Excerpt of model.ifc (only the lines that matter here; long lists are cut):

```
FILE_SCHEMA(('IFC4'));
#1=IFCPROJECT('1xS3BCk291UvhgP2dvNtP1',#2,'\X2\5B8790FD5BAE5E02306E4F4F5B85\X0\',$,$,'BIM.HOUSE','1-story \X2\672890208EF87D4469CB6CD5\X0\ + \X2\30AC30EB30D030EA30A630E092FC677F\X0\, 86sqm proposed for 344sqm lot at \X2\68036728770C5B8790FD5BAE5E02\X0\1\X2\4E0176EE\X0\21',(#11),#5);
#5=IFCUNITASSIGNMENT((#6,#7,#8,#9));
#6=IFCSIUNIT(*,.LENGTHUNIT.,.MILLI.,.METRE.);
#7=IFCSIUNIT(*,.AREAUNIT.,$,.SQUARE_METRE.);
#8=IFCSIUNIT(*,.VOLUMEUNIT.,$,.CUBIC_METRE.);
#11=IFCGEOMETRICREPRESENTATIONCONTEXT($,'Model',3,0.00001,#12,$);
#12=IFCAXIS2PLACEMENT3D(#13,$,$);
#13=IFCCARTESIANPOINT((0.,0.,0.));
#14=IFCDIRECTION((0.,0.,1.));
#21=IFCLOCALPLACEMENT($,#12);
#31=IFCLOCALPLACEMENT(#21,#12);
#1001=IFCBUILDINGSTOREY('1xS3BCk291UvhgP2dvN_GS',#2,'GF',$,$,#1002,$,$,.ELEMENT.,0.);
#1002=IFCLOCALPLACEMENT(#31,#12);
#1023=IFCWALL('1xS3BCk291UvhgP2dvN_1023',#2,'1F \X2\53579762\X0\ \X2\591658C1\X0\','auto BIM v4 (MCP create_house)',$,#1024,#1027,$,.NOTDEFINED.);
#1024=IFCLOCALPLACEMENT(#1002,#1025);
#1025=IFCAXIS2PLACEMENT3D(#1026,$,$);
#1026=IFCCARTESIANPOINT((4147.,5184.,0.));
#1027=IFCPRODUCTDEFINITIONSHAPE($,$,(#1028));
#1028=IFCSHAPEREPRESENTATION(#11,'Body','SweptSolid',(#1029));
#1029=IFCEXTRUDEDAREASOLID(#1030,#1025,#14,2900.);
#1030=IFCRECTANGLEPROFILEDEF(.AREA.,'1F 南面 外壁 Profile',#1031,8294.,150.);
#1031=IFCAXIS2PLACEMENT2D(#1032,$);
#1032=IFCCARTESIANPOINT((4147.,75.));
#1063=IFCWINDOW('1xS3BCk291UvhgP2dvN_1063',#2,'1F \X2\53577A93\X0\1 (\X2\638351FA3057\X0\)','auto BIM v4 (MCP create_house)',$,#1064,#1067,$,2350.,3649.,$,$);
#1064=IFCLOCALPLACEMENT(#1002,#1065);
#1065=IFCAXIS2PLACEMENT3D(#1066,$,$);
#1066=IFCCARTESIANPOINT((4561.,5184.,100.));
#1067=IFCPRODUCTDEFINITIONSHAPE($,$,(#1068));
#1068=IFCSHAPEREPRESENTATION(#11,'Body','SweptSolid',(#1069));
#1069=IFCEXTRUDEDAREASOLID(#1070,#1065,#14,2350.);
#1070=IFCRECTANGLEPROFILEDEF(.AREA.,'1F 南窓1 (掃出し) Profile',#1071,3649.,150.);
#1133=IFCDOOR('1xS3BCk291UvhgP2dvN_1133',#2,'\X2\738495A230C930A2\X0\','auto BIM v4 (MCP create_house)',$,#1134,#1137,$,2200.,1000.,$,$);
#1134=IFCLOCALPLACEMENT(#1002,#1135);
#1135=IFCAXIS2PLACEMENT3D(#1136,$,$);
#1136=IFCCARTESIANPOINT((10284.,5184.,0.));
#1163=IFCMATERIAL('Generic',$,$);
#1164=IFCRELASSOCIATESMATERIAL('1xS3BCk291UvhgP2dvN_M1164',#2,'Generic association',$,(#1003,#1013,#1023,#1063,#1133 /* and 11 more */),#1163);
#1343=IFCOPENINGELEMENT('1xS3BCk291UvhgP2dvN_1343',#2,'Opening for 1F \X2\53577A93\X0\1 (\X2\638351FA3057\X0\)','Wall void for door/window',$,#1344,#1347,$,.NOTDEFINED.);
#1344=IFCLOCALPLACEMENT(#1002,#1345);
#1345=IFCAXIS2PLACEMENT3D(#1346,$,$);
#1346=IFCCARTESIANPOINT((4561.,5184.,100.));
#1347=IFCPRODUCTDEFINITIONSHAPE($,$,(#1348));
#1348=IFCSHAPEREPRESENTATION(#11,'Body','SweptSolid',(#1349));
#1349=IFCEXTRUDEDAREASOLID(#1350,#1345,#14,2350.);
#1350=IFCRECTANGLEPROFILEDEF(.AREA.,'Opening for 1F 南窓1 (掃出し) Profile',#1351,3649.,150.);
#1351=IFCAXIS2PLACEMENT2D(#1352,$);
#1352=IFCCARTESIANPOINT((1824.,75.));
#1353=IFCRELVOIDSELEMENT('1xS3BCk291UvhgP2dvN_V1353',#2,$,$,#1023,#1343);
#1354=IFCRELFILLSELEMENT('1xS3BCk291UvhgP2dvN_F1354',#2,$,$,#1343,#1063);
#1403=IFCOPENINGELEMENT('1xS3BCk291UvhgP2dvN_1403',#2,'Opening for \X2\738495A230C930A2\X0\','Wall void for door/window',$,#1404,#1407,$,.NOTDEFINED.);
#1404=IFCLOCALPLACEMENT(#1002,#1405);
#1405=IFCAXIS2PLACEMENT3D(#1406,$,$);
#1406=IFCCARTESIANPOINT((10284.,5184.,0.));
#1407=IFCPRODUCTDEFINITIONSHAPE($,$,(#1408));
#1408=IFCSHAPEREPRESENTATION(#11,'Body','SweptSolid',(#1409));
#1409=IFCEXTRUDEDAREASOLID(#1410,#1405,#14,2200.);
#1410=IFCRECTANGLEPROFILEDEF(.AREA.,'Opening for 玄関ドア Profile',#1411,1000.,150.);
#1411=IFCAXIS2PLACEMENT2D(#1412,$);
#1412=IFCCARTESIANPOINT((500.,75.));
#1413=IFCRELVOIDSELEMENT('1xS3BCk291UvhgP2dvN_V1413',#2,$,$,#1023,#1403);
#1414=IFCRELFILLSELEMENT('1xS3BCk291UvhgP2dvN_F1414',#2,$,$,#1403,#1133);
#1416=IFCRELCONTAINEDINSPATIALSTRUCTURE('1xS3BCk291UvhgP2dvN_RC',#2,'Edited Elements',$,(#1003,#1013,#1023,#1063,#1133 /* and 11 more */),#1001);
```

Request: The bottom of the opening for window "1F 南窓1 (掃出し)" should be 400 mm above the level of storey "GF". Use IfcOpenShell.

```python
import numpy as np
import ifcopenshell
import ifcopenshell.api.geometry
import ifcopenshell.geom
import ifcopenshell.util.element
import ifcopenshell.util.placement
import ifcopenshell.util.shape
import ifcopenshell.util.unit

model = ifcopenshell.open("model.ifc")
unit_scale = ifcopenshell.util.unit.calculate_unit_scale(model)

window = model.by_guid("1xS3BCk291UvhgP2dvN_1063")
opening = window.FillsVoids[0].RelatingOpeningElement
storey = ifcopenshell.util.element.get_container(window, ifc_class="IfcBuildingStorey")
level = ifcopenshell.util.placement.get_local_placement(storey.ObjectPlacement)[2, 3]

# The opening's origin need not be at the sill, so measure its lowest point.
shape = ifcopenshell.geom.create_shape(ifcopenshell.geom.settings(), opening)
bottom = ifcopenshell.util.shape.get_shape_bottom_elevation(shape, shape.geometry) / unit_scale
dz = level + 0.4 / unit_scale - bottom

shift = np.array([0.0, 0.0, dz])
# The window is not placed relative to its opening, so move both.
for product in (opening, window):
    matrix = ifcopenshell.util.placement.get_local_placement(product.ObjectPlacement)
    matrix[:3, 3] += shift
    ifcopenshell.api.geometry.edit_object_placement(model, product=product, matrix=matrix, is_si=False)

print(f"moved by {dz * unit_scale:+.3f} m")

model.write("model-out.ifc")
```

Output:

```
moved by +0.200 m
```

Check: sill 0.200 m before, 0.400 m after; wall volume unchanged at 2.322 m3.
